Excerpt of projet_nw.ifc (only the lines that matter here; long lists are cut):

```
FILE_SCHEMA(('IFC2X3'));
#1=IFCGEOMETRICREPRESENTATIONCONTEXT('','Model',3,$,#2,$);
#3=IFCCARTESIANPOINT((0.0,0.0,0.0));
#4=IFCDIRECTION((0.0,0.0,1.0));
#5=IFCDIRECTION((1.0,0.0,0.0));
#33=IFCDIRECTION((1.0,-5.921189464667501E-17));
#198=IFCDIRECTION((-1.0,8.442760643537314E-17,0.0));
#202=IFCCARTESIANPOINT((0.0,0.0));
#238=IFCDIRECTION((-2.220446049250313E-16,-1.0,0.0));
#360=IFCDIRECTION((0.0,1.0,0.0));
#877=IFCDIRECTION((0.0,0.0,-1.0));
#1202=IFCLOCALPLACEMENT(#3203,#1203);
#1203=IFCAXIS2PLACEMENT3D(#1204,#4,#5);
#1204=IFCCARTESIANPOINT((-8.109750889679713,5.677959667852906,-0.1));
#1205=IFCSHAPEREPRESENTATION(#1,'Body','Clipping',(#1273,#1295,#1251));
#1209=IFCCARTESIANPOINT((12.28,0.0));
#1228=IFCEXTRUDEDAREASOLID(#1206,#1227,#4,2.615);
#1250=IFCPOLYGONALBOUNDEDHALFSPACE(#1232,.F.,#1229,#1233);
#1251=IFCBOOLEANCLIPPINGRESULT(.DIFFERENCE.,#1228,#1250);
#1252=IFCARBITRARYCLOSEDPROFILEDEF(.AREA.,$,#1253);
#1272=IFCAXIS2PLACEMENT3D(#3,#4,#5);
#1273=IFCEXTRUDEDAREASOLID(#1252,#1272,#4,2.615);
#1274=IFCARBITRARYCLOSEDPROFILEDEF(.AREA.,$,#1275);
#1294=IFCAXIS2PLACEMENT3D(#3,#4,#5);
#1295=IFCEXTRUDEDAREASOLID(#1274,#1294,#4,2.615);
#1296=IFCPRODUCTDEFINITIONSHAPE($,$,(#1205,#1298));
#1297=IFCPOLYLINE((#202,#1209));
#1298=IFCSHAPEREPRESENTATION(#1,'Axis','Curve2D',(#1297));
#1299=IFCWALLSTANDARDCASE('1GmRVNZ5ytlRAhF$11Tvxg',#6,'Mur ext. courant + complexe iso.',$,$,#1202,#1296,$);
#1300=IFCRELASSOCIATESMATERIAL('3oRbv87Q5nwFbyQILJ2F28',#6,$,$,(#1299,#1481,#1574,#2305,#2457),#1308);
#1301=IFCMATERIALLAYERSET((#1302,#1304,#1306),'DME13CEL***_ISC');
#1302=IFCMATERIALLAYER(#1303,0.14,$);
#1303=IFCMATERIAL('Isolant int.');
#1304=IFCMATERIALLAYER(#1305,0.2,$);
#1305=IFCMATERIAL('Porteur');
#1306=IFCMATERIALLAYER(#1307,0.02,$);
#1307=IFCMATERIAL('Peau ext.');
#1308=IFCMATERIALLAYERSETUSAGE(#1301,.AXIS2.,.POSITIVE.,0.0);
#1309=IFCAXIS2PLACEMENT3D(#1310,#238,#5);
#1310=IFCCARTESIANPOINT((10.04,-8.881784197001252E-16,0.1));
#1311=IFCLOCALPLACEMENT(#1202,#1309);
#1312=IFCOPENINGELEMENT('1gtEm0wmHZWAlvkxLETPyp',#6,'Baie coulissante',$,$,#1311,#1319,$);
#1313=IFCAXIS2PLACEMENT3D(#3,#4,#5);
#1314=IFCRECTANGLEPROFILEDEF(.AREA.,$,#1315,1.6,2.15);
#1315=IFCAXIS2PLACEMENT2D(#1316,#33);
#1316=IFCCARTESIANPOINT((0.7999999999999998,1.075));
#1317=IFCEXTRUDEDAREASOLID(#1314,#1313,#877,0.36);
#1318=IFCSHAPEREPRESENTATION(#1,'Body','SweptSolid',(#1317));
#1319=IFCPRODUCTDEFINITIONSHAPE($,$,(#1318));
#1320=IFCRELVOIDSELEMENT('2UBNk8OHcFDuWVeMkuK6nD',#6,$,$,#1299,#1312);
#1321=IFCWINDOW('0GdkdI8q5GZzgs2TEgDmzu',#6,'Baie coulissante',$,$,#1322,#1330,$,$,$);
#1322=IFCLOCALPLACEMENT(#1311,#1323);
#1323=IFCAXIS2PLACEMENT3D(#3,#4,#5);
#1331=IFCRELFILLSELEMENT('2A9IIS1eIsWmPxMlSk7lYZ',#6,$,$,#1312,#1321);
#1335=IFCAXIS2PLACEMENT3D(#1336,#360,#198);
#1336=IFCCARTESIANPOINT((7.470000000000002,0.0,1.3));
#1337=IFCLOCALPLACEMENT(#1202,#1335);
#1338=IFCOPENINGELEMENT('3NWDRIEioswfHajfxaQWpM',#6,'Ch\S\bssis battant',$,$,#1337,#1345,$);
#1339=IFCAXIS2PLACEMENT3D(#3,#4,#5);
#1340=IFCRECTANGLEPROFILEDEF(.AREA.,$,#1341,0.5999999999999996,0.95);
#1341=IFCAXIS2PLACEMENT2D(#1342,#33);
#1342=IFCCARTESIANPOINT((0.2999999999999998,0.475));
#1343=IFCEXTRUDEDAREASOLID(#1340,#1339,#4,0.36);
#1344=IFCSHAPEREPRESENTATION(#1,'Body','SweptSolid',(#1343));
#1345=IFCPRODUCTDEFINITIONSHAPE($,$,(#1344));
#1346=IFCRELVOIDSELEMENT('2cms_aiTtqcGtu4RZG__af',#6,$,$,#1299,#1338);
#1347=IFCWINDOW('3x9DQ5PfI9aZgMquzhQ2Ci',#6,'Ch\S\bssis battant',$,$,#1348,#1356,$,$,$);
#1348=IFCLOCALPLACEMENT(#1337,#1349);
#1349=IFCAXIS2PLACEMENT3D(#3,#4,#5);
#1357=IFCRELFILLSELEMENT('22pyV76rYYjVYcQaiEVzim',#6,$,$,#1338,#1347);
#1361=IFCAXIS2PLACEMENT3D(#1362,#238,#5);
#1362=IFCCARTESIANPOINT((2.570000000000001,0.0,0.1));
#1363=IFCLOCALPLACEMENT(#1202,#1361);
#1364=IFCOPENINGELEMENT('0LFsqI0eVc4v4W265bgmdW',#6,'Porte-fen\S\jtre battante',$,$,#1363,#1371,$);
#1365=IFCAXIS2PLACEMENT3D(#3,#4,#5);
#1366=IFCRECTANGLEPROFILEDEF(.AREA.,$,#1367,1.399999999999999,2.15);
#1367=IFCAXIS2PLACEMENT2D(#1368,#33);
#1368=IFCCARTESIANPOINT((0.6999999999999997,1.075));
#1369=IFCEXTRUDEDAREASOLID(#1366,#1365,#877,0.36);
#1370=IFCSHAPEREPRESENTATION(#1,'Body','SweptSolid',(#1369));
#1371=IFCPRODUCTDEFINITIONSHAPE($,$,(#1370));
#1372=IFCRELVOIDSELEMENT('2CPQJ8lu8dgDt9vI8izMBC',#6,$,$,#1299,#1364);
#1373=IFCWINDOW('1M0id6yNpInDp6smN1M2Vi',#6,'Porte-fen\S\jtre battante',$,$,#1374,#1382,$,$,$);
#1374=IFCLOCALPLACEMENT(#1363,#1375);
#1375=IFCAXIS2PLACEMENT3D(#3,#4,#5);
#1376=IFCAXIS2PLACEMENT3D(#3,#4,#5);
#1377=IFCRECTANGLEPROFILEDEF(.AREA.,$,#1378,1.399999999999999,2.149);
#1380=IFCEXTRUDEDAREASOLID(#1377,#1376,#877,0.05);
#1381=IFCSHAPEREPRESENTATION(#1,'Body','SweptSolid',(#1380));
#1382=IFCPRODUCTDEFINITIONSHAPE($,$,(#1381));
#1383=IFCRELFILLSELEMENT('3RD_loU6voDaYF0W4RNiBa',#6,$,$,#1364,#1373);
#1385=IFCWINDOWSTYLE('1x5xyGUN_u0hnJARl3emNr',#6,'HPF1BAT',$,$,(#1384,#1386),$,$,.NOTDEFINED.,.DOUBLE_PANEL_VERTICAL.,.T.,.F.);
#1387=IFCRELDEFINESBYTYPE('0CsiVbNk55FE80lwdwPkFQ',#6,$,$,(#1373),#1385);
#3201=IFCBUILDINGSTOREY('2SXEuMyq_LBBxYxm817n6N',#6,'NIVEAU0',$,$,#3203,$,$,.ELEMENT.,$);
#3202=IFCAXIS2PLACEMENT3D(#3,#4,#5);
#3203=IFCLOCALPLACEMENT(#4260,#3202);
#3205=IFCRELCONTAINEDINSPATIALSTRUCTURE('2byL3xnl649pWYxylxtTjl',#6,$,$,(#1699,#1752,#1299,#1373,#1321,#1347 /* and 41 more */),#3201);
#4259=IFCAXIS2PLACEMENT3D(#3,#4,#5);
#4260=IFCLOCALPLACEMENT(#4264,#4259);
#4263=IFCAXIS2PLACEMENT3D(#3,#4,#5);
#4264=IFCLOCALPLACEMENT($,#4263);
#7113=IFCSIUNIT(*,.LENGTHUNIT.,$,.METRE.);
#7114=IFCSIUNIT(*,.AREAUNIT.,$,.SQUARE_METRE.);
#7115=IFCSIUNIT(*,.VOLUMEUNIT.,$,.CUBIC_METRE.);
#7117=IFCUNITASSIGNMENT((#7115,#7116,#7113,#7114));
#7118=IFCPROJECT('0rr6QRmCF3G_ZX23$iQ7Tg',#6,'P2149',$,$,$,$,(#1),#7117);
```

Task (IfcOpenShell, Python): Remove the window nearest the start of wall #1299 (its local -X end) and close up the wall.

```python
import ifcopenshell
import ifcopenshell.api.feature
import ifcopenshell.api.root
import ifcopenshell.geom
import ifcopenshell.util.shape

model = ifcopenshell.open("projet_nw.ifc")
settings = ifcopenshell.geom.settings()


def volume(element):
    """Net volume in cubic metres, openings subtracted."""
    shape = ifcopenshell.geom.create_shape(settings, element)
    return ifcopenshell.util.shape.get_volume(shape.geometry)


window = model.by_guid("1M0id6yNpInDp6smN1M2Vi")
opening = window.FillsVoids[0].RelatingOpeningElement
wall = opening.VoidsElements[0].RelatingBuildingElement
before = volume(wall)

ifcopenshell.api.root.remove_product(model, product=window)
ifcopenshell.api.feature.remove_feature(model, feature=opening)

after = volume(wall)

print(f"wall volume {before:.3f} -> {after:.3f} m3")

model.write("projet_nw_rev.ifc")
```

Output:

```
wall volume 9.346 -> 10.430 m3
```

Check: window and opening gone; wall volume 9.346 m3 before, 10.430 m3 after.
